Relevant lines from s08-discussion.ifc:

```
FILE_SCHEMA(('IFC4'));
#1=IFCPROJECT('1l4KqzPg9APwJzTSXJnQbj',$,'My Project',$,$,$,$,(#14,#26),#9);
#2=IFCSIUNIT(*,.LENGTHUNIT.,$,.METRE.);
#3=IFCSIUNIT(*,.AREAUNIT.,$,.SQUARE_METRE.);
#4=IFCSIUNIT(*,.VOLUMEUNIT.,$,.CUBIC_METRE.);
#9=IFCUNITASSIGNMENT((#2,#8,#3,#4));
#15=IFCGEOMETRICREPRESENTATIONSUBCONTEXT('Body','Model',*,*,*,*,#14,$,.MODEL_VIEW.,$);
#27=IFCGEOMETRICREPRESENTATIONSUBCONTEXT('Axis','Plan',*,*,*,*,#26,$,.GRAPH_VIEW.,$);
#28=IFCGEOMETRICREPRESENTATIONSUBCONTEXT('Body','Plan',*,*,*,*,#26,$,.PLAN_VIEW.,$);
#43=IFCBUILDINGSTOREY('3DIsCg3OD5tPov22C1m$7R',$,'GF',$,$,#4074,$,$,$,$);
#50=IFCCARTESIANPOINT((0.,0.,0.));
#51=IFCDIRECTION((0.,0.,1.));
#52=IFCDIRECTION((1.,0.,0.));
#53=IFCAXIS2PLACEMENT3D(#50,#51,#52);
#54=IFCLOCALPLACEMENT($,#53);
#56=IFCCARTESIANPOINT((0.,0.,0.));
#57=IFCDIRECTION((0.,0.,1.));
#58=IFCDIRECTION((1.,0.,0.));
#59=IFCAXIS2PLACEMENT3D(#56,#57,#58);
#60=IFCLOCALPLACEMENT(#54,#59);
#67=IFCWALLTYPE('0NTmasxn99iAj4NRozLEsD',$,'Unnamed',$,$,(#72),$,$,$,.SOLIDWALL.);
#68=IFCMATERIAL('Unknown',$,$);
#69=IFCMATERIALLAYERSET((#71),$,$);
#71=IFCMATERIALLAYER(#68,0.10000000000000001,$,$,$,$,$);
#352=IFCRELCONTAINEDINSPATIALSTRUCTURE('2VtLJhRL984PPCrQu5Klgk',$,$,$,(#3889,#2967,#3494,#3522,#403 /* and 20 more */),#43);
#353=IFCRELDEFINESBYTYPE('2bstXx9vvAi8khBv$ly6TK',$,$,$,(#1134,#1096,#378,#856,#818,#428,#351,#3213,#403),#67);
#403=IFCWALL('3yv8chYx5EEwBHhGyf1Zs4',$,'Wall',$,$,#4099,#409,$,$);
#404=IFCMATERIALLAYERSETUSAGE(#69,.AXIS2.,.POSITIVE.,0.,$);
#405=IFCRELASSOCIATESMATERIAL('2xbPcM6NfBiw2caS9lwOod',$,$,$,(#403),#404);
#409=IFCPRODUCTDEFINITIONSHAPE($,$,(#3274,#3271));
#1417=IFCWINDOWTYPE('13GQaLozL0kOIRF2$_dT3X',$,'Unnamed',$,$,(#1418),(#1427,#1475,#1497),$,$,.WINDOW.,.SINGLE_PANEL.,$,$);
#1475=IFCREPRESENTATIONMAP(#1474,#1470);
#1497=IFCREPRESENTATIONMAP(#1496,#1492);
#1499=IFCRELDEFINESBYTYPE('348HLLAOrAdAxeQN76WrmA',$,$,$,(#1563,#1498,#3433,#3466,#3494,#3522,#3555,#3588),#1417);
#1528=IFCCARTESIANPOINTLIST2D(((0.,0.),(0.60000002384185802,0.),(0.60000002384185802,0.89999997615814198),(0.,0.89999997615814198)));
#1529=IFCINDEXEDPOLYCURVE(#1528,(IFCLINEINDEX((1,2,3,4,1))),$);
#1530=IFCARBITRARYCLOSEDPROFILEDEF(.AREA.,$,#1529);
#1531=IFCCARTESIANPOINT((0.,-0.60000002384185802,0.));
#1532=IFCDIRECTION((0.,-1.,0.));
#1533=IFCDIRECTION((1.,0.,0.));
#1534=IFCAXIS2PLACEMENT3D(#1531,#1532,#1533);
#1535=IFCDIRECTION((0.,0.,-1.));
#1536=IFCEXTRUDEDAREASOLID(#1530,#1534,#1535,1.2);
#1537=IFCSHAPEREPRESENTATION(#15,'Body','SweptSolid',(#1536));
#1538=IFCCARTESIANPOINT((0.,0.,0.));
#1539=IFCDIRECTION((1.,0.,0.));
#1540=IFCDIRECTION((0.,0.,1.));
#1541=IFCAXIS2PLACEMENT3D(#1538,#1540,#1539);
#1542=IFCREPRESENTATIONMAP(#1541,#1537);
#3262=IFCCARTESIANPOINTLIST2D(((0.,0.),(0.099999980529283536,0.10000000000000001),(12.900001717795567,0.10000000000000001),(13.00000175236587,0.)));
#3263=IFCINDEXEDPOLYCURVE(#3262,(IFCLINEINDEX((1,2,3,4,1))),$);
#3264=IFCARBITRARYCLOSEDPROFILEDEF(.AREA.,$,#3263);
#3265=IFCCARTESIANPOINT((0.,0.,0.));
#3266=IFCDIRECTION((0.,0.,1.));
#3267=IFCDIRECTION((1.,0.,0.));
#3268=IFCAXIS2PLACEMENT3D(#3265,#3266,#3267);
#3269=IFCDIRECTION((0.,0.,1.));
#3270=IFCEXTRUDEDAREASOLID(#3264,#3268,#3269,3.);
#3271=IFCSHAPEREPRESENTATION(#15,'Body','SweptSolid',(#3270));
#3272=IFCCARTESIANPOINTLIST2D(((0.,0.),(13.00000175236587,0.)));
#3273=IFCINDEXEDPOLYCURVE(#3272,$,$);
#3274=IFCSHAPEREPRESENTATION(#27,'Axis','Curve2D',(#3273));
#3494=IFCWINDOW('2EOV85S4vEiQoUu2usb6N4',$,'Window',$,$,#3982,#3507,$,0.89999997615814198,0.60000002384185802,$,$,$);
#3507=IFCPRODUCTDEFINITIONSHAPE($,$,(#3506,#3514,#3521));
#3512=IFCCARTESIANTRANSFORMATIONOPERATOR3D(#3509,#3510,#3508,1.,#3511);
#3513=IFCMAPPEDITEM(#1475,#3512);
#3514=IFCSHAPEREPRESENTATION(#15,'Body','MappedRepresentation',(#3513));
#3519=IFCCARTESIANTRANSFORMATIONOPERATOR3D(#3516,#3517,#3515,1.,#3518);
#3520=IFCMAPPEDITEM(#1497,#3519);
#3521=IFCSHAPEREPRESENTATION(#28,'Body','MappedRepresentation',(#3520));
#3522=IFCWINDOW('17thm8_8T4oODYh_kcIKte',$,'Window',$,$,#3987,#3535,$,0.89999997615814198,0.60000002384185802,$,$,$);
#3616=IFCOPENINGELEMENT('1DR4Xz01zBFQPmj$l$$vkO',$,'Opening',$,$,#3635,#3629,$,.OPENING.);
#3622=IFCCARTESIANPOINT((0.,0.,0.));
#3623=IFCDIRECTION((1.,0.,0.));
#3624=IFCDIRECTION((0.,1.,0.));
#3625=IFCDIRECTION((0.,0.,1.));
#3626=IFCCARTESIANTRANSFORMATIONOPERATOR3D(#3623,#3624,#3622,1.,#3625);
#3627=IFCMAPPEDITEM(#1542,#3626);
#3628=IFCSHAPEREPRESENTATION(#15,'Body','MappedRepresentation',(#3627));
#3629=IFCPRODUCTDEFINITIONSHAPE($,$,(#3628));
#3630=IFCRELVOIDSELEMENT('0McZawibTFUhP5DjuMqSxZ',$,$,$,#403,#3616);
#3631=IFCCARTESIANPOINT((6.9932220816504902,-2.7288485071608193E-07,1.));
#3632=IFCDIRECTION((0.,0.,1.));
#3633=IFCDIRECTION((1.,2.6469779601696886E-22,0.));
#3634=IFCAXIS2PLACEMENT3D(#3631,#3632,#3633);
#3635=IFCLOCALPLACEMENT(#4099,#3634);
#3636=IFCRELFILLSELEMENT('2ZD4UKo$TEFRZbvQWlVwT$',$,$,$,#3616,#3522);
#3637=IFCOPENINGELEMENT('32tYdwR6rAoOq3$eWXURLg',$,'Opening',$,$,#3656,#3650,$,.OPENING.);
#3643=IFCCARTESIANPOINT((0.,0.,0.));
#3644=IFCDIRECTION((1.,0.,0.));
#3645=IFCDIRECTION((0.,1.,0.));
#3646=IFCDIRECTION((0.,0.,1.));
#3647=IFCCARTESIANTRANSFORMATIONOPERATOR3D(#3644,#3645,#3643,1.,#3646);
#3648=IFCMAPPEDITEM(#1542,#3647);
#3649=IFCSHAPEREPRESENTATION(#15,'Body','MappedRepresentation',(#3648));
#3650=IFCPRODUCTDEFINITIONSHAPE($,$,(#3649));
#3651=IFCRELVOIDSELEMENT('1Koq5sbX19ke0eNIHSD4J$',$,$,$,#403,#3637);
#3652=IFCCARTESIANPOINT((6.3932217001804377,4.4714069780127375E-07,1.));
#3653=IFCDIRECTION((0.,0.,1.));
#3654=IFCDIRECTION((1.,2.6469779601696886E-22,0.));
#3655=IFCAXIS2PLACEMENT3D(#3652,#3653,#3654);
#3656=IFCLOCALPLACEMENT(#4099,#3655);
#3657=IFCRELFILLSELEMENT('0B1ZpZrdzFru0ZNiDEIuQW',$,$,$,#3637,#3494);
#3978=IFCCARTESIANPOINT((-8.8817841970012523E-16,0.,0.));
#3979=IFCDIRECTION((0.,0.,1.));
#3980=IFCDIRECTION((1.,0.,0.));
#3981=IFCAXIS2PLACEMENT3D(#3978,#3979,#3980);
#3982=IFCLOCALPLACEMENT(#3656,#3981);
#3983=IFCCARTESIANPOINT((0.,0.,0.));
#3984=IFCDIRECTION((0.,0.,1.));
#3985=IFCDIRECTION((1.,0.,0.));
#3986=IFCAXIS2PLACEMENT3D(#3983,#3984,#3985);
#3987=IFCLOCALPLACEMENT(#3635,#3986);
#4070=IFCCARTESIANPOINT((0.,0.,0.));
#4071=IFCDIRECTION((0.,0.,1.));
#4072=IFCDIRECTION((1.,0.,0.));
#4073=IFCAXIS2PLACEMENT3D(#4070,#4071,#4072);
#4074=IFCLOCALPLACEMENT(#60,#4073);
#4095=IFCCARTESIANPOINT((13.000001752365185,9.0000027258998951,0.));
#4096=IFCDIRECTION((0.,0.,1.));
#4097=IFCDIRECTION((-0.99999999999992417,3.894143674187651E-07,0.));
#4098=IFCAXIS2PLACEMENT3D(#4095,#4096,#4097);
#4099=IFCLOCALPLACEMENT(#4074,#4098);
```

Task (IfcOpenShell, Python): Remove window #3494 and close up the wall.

```python
import ifcopenshell
import ifcopenshell.api.feature
import ifcopenshell.api.root
import ifcopenshell.geom
import ifcopenshell.util.shape

model = ifcopenshell.open("s08-discussion.ifc")
settings = ifcopenshell.geom.settings()


def volume(element):
    """Net volume in cubic metres, openings subtracted."""
    shape = ifcopenshell.geom.create_shape(settings, element)
    return ifcopenshell.util.shape.get_volume(shape.geometry)


window = model.by_id(3494)
opening = window.FillsVoids[0].RelatingOpeningElement
wall = opening.VoidsElements[0].RelatingBuildingElement
before = volume(wall)

ifcopenshell.api.root.remove_product(model, product=window)
ifcopenshell.api.feature.remove_feature(model, feature=opening)

after = volume(wall)

print(f"wall volume {before:.3f} -> {after:.3f} m3")

model.write("s08-discussion_v2.ifc")
```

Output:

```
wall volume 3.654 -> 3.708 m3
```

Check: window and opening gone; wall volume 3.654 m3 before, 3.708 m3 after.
